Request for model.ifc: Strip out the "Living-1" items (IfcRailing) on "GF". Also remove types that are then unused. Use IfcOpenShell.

First a look at what the model holds.

```python
import ifcopenshell
import ifcopenshell.util.element

model = ifcopenshell.open("model.ifc")
print(model.schema)
storey = next(s for s in model.by_type("IfcBuildingStorey") if s.Name == "GF")
railings = [e for e in ifcopenshell.util.element.get_decomposition(storey) if e.is_a("IfcRailing")]
seen = {}
for e in railings:
    element_type = ifcopenshell.util.element.get_type(e)
    name = element_type.Name if element_type not in (None, e) else None
    seen[name] = seen.get(name, 0) + 1
for name, count in sorted(seen.items(), key=str):
    print(count, "x", name)
```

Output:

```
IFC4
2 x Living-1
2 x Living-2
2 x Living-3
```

```python
import ifcopenshell
import ifcopenshell.api.root
import ifcopenshell.util.element

model = ifcopenshell.open("model.ifc")

storey = next(s for s in model.by_type("IfcBuildingStorey") if s.Name == "GF")
railings = [e for e in ifcopenshell.util.element.get_decomposition(storey) if e.is_a("IfcRailing")]
targets = [e for e in railings if (t := ifcopenshell.util.element.get_type(e)) not in (None, e) and t.Name == "Living-1"]
types = {ifcopenshell.util.element.get_type(e) for e in targets} - {None, *targets}

for e in targets:
    ifcopenshell.api.root.remove_product(model, product=e)
print(len(targets), "removed")

unused = [t for t in types if not ifcopenshell.util.element.get_types(t)]
for t in unused:
    ifcopenshell.api.root.remove_product(model, product=t)
print(len(unused), "unused types removed")

model.write("model_rev.ifc")
```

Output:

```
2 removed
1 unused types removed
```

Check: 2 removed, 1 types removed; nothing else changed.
